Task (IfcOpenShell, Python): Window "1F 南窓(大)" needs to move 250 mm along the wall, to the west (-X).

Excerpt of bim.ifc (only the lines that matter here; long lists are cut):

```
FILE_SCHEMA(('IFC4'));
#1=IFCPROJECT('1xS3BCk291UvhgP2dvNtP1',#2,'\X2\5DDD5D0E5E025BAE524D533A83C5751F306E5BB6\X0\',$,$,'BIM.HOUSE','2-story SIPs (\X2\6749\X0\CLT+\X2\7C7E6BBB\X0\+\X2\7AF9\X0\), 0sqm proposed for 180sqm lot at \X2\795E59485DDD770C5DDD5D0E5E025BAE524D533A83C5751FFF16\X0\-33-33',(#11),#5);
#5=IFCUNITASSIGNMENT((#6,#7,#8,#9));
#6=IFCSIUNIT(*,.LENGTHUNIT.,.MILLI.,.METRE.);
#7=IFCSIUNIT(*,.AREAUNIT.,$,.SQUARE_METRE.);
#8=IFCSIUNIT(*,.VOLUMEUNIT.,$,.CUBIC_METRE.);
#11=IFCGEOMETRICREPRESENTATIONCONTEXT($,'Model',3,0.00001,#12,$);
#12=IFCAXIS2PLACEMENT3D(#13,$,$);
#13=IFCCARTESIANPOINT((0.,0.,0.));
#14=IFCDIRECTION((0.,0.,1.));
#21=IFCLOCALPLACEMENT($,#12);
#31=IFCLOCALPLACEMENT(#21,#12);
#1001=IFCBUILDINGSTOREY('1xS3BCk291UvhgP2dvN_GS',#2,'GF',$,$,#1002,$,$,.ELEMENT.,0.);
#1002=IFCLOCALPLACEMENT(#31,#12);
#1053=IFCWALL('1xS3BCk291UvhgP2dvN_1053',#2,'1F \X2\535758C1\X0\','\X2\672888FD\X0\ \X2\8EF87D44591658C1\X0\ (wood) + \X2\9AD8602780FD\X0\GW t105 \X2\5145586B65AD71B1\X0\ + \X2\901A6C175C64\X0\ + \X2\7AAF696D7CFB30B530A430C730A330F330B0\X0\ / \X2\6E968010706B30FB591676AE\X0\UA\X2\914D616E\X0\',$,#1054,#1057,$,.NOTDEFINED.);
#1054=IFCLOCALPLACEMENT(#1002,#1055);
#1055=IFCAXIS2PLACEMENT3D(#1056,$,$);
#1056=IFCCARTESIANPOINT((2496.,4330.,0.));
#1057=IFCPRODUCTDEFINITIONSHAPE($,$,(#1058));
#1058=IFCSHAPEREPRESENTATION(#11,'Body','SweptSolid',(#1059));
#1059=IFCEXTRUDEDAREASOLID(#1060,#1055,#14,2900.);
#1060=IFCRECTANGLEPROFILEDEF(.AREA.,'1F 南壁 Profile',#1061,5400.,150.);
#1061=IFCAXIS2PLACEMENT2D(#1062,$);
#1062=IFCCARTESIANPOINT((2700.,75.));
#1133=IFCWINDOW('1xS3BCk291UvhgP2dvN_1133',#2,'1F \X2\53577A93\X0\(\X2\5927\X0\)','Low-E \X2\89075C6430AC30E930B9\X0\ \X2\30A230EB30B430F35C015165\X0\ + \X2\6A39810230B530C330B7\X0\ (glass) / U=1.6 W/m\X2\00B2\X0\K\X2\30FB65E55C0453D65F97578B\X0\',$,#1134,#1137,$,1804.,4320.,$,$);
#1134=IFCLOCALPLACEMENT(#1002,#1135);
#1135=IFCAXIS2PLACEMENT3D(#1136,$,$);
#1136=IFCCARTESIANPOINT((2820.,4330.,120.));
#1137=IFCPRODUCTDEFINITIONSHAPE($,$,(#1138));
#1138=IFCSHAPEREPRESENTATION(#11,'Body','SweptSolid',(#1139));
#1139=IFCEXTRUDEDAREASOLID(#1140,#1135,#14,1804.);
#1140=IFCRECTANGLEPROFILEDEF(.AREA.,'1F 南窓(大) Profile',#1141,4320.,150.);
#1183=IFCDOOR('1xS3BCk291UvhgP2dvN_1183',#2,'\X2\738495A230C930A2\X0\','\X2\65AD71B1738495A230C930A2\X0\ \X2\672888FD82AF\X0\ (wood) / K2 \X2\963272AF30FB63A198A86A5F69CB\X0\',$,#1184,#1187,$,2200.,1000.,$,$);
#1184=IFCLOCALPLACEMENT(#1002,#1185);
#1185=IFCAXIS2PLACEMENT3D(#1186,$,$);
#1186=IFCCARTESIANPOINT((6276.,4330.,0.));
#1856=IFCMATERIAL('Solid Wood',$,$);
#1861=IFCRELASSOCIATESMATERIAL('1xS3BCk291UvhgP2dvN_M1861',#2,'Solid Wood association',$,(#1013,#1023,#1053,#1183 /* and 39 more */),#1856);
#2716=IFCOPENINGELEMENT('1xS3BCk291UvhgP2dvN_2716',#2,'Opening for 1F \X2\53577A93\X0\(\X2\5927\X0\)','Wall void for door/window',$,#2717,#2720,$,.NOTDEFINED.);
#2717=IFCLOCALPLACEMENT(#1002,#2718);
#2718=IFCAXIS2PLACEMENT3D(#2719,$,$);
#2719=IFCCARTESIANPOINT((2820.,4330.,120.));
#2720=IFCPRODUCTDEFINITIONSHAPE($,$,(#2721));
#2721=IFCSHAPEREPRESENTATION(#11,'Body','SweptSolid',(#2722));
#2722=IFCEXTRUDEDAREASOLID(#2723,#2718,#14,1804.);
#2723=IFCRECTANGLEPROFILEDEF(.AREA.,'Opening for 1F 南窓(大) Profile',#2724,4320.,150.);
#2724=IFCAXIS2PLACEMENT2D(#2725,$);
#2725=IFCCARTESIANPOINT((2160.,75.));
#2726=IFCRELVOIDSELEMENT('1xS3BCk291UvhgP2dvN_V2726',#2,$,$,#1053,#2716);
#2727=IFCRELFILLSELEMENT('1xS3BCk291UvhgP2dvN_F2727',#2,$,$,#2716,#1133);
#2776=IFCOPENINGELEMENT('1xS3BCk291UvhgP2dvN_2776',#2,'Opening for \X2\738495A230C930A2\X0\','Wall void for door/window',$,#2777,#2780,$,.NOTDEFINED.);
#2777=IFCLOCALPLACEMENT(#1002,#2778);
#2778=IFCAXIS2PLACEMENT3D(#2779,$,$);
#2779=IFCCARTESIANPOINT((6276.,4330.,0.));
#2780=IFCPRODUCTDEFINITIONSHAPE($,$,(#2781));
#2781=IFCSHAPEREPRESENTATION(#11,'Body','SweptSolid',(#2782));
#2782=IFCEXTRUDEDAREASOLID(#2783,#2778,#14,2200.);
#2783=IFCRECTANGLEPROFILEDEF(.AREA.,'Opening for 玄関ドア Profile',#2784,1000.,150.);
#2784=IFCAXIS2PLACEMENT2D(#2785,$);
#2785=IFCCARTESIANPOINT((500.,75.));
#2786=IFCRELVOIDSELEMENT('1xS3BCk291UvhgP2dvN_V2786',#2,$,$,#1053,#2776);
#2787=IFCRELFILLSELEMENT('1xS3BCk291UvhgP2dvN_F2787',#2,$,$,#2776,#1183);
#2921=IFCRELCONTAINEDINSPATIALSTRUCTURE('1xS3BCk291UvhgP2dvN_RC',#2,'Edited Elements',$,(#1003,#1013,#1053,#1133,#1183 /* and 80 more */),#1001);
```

```python
import ifcopenshell
import ifcopenshell.api.geometry
import ifcopenshell.util.placement

model = ifcopenshell.open("bim.ifc")

window = model.by_guid("1xS3BCk291UvhgP2dvN_1133")
opening = window.FillsVoids[0].RelatingOpeningElement
wall = opening.VoidsElements[0].RelatingBuildingElement

wall_matrix = ifcopenshell.util.placement.get_local_placement(wall.ObjectPlacement)
shift = wall_matrix[:3, 0] * -250.0
before = ifcopenshell.util.placement.get_local_placement(window.ObjectPlacement)[:3, 3].copy()

# The window is not placed relative to its opening, so move both.
for product in (opening, window):
    matrix = ifcopenshell.util.placement.get_local_placement(product.ObjectPlacement)
    matrix[:3, 3] += shift
    ifcopenshell.api.geometry.edit_object_placement(model, product=product, matrix=matrix, is_si=False)

after = ifcopenshell.util.placement.get_local_placement(window.ObjectPlacement)[:3, 3]
print("window moved by", (after - before).round(3) + 0.0)

model.write("bim_v2.ifc")
```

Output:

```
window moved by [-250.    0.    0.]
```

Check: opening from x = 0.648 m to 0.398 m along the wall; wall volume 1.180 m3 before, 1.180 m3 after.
